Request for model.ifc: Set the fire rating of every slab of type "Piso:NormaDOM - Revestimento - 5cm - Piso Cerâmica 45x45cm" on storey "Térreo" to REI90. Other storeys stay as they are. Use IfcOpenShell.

First a look at what the model holds.

```python
import ifcopenshell
import ifcopenshell.util.element

model = ifcopenshell.open("model.ifc")
print(model.schema)
storey = next(s for s in model.by_type("IfcBuildingStorey") if s.Name == "Térreo")
slabs = [e for e in ifcopenshell.util.element.get_decomposition(storey) if e.is_a("IfcSlab")]
seen = {}
for e in slabs:
    element_type = ifcopenshell.util.element.get_type(e)
    key = (element_type.Name if element_type != e and element_type else None, ifcopenshell.util.element.get_pset(e, "Pset_SlabCommon", "FireRating"))
    seen[key] = seen.get(key, 0) + 1
for (name, value), count in sorted(seen.items(), key=str):
    print(count, "x", name, "|", value)
```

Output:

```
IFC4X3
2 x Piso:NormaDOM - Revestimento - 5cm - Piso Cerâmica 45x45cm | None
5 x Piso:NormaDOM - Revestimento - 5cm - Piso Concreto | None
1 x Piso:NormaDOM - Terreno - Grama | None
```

```python
import ifcopenshell
import ifcopenshell.api.pset
import ifcopenshell.util.element

model = ifcopenshell.open("model.ifc")

storey = next(s for s in model.by_type("IfcBuildingStorey") if s.Name == "Térreo")
slabs = [e for e in ifcopenshell.util.element.get_decomposition(storey) if e.is_a("IfcSlab")]

count = 0
for e in slabs:
    element_type = ifcopenshell.util.element.get_type(e)
    if element_type in (None, e) or element_type.Name != "Piso:NormaDOM - Revestimento - 5cm - Piso Cerâmica 45x45cm":
        continue
    # add_pset returns the element's existing set when there is one.
    pset = ifcopenshell.api.pset.add_pset(model, product=e, name="Pset_SlabCommon")
    ifcopenshell.api.pset.edit_pset(model, pset=pset, properties={"FireRating": "REI90"})
    count += 1

print(count, "slabs updated")

model.write("model_updated.ifc")
```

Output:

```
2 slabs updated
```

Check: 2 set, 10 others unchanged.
